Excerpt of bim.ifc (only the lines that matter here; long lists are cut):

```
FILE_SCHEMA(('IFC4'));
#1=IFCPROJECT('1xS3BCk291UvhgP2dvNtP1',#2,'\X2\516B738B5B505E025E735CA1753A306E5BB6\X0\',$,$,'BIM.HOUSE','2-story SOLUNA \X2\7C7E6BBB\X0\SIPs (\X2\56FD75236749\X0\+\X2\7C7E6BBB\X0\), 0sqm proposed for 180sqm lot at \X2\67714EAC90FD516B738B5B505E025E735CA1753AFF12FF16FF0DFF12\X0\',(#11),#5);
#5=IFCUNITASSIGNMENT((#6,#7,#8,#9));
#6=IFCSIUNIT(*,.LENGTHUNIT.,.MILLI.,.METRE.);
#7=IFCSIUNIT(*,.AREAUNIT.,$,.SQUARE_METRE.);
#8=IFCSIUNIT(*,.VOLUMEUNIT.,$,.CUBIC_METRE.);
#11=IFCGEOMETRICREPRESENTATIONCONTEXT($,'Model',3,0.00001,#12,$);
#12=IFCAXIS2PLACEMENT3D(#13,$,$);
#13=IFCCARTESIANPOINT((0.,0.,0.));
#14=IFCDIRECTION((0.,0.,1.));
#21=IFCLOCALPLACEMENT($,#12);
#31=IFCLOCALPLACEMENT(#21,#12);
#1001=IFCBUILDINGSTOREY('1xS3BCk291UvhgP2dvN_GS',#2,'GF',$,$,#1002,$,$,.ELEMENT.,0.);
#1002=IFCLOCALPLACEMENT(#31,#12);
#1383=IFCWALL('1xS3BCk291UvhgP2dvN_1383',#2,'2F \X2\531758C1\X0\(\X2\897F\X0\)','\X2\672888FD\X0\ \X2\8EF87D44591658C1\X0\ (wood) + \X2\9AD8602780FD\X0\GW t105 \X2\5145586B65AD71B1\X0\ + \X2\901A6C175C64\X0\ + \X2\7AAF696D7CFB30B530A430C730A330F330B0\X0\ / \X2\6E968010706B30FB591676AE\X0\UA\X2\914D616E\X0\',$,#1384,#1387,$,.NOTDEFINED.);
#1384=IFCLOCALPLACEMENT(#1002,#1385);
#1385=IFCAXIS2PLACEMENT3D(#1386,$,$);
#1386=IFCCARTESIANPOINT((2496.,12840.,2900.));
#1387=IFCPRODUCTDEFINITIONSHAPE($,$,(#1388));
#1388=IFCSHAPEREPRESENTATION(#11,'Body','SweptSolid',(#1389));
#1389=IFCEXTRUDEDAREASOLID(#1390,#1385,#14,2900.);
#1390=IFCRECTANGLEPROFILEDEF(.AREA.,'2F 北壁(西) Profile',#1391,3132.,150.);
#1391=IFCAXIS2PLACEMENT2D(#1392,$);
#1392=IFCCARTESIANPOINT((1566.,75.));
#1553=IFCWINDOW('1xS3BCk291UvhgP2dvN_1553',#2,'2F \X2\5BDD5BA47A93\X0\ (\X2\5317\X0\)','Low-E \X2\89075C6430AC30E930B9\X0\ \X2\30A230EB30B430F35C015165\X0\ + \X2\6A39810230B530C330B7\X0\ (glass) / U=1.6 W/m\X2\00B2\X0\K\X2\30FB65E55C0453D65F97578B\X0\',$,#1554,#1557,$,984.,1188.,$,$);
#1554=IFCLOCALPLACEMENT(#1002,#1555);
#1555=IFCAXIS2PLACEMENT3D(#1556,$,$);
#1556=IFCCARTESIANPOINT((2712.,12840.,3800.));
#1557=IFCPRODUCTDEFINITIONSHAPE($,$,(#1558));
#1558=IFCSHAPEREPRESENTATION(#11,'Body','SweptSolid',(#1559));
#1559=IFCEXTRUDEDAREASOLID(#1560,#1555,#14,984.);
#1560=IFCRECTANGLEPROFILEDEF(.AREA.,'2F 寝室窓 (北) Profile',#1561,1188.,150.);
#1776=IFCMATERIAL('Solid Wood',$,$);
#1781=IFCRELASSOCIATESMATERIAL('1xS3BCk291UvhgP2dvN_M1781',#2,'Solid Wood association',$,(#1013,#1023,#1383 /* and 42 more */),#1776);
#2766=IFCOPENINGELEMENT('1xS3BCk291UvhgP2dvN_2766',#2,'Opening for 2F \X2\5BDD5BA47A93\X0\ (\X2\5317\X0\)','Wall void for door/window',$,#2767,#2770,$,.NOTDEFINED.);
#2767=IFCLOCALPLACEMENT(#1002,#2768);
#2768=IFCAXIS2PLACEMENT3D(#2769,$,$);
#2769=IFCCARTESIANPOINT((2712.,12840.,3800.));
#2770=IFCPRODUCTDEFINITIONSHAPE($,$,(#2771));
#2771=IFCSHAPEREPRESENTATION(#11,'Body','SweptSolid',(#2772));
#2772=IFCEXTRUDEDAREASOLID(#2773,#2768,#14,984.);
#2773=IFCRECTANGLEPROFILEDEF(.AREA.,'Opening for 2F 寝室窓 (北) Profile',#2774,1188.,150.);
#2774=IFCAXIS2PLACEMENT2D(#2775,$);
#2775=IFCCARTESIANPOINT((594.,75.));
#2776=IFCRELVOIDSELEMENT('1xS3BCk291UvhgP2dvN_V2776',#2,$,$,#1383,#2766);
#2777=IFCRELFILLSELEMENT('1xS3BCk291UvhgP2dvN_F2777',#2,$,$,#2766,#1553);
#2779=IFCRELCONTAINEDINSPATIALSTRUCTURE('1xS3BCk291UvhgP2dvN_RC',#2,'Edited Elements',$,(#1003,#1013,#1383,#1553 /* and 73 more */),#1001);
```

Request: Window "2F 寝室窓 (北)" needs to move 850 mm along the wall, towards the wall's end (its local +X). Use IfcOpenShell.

```python
import ifcopenshell
import ifcopenshell.api.geometry
import ifcopenshell.util.placement
import ifcopenshell.util.unit

model = ifcopenshell.open("bim.ifc")
unit_scale = ifcopenshell.util.unit.calculate_unit_scale(model)

window = model.by_guid("1xS3BCk291UvhgP2dvN_1553")
opening = window.FillsVoids[0].RelatingOpeningElement
wall = opening.VoidsElements[0].RelatingBuildingElement

wall_matrix = ifcopenshell.util.placement.get_local_placement(wall.ObjectPlacement)
shift = wall_matrix[:3, 0] * 0.85 / unit_scale
before = ifcopenshell.util.placement.get_local_placement(window.ObjectPlacement)[:3, 3].copy()

# The window is not placed relative to its opening, so move both.
for product in (opening, window):
    matrix = ifcopenshell.util.placement.get_local_placement(product.ObjectPlacement)
    matrix[:3, 3] += shift
    ifcopenshell.api.geometry.edit_object_placement(model, product=product, matrix=matrix, is_si=False)

after = ifcopenshell.util.placement.get_local_placement(window.ObjectPlacement)[:3, 3]
print("window moved by", (after - before).round(3) + 0.0)

model.write("bim_rev.ifc")
```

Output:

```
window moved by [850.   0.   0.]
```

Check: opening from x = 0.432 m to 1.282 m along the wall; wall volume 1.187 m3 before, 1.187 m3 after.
